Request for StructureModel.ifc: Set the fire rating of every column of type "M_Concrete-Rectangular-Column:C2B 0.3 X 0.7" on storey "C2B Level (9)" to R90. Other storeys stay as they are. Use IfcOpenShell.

First a look at what the model holds.

```python
import ifcopenshell
import ifcopenshell.util.element

model = ifcopenshell.open("StructureModel.ifc")
print(model.schema)
storey = next(s for s in model.by_type("IfcBuildingStorey") if s.Name == "C2B Level (9)")
columns = [e for e in ifcopenshell.util.element.get_decomposition(storey) if e.is_a("IfcColumn")]
seen = {}
for e in columns:
    element_type = ifcopenshell.util.element.get_type(e)
    key = (element_type.Name if element_type != e and element_type else None, ifcopenshell.util.element.get_pset(e, "Pset_ColumnCommon", "FireRating"))
    seen[key] = seen.get(key, 0) + 1
for (name, value), count in sorted(seen.items(), key=str):
    print(count, "x", name, "|", value)
```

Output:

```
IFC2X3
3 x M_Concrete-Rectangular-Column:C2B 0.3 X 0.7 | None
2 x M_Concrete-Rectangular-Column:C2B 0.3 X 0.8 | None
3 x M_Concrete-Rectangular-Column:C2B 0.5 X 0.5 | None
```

```python
import ifcopenshell
import ifcopenshell.api.pset
import ifcopenshell.util.element

model = ifcopenshell.open("StructureModel.ifc")

storey = next(s for s in model.by_type("IfcBuildingStorey") if s.Name == "C2B Level (9)")
columns = [e for e in ifcopenshell.util.element.get_decomposition(storey) if e.is_a("IfcColumn")]

count = 0
for e in columns:
    element_type = ifcopenshell.util.element.get_type(e)
    if element_type in (None, e) or element_type.Name != "M_Concrete-Rectangular-Column:C2B 0.3 X 0.7":
        continue
    # add_pset returns the element's existing set when there is one.
    pset = ifcopenshell.api.pset.add_pset(model, product=e, name="Pset_ColumnCommon")
    ifcopenshell.api.pset.edit_pset(model, pset=pset, properties={"FireRating": "R90"})
    count += 1

print(count, "columns updated")

model.write("StructureModel_v2.ifc")
```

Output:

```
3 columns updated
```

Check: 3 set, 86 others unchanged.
